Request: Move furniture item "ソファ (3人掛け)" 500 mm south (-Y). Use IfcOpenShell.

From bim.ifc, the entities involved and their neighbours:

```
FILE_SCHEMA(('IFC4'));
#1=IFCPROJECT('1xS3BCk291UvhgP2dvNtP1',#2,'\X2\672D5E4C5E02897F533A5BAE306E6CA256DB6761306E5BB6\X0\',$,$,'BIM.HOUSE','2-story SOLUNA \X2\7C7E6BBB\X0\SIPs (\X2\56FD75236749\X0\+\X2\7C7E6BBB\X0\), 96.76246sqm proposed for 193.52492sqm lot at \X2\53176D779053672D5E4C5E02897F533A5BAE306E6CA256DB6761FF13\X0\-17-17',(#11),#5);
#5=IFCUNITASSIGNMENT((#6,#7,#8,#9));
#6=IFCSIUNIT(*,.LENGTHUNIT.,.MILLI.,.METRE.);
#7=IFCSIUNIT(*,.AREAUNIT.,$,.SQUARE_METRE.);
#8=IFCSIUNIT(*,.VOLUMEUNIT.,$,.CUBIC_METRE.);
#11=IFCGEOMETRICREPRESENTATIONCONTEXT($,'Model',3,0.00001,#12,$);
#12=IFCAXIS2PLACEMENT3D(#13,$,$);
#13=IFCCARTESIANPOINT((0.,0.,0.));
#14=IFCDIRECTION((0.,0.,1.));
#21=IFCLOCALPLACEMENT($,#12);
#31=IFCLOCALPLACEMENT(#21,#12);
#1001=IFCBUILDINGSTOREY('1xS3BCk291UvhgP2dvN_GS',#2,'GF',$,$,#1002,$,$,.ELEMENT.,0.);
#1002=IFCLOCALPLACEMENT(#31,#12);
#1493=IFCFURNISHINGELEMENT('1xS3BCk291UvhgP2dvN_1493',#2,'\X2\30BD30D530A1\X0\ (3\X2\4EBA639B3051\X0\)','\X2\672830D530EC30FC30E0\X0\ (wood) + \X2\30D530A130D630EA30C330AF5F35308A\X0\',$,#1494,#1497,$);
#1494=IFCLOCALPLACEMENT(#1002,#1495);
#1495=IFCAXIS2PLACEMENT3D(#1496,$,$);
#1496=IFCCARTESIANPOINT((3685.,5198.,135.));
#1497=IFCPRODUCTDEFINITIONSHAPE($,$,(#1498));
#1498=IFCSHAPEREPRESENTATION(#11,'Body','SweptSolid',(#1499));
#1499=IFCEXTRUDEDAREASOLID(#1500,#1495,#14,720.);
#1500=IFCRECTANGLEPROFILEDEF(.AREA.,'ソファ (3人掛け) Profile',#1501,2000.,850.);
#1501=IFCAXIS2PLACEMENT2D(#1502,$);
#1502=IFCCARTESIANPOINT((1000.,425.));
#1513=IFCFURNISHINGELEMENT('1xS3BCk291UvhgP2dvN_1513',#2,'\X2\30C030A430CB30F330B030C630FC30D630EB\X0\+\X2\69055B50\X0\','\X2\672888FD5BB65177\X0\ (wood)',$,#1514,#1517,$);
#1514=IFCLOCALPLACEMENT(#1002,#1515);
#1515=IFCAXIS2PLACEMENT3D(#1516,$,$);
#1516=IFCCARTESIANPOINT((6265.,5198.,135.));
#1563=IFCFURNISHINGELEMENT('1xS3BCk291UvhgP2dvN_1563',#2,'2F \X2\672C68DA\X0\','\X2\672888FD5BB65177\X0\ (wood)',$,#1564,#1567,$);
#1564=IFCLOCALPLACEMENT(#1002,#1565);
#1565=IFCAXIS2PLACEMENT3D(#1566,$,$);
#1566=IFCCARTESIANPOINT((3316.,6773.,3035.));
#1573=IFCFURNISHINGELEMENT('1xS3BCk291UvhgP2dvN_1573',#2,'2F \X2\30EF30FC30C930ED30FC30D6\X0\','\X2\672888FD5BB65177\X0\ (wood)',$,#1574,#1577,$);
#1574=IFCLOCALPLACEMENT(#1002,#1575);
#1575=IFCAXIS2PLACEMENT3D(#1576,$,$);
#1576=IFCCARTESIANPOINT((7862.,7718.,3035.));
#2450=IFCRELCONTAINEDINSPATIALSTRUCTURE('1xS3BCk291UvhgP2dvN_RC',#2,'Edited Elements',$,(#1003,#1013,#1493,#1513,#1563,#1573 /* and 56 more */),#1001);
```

```python
import ifcopenshell
import ifcopenshell.api.geometry
import ifcopenshell.util.placement
import ifcopenshell.util.unit

model = ifcopenshell.open("bim.ifc")
unit_scale = ifcopenshell.util.unit.calculate_unit_scale(model)

item = model.by_id(1493)
matrix = ifcopenshell.util.placement.get_local_placement(item.ObjectPlacement)
matrix[1, 3] -= 0.5 / unit_scale
ifcopenshell.api.geometry.edit_object_placement(model, product=item, matrix=matrix, is_si=False)

print(ifcopenshell.util.placement.get_local_placement(item.ObjectPlacement).round(3) + 0.0)

model.write("bim_updated.ifc")
```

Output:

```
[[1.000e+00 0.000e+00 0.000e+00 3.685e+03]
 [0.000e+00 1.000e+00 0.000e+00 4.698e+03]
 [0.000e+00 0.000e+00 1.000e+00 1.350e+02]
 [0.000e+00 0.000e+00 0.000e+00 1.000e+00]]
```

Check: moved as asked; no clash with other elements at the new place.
